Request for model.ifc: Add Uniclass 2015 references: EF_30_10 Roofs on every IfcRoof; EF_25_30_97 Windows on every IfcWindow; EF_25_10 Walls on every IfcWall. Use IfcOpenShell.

First a look at what the model holds.

```python
import ifcopenshell

model = ifcopenshell.open("model.ifc")
print(model.schema)
print("classifications:", [c.Name for c in model.by_type("IfcClassification")])
for ifc_class in ("IfcDoor", "IfcRoof", "IfcStair", "IfcWall", "IfcWindow"):
    print(ifc_class, len(model.by_type(ifc_class)))
```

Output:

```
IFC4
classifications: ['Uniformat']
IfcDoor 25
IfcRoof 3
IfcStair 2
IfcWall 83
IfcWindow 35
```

```python
import ifcopenshell
import ifcopenshell.api.classification

model = ifcopenshell.open("model.ifc")

system = ifcopenshell.api.classification.add_classification(model, classification="Uniclass 2015")

codes = {
    "IfcRoof": ("EF_30_10", "Roofs"),
    "IfcWindow": ("EF_25_30_97", "Windows"),
    "IfcWall": ("EF_25_10", "Walls"),
}
for ifc_class, (code, name) in codes.items():
    products = model.by_type(ifc_class)
    ifcopenshell.api.classification.add_reference(
        model, products=products, classification=system, identification=code, name=name
    )
    print(code, len(products))

model.write("model_rev.ifc")
```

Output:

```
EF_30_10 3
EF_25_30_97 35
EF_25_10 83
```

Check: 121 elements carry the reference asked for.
